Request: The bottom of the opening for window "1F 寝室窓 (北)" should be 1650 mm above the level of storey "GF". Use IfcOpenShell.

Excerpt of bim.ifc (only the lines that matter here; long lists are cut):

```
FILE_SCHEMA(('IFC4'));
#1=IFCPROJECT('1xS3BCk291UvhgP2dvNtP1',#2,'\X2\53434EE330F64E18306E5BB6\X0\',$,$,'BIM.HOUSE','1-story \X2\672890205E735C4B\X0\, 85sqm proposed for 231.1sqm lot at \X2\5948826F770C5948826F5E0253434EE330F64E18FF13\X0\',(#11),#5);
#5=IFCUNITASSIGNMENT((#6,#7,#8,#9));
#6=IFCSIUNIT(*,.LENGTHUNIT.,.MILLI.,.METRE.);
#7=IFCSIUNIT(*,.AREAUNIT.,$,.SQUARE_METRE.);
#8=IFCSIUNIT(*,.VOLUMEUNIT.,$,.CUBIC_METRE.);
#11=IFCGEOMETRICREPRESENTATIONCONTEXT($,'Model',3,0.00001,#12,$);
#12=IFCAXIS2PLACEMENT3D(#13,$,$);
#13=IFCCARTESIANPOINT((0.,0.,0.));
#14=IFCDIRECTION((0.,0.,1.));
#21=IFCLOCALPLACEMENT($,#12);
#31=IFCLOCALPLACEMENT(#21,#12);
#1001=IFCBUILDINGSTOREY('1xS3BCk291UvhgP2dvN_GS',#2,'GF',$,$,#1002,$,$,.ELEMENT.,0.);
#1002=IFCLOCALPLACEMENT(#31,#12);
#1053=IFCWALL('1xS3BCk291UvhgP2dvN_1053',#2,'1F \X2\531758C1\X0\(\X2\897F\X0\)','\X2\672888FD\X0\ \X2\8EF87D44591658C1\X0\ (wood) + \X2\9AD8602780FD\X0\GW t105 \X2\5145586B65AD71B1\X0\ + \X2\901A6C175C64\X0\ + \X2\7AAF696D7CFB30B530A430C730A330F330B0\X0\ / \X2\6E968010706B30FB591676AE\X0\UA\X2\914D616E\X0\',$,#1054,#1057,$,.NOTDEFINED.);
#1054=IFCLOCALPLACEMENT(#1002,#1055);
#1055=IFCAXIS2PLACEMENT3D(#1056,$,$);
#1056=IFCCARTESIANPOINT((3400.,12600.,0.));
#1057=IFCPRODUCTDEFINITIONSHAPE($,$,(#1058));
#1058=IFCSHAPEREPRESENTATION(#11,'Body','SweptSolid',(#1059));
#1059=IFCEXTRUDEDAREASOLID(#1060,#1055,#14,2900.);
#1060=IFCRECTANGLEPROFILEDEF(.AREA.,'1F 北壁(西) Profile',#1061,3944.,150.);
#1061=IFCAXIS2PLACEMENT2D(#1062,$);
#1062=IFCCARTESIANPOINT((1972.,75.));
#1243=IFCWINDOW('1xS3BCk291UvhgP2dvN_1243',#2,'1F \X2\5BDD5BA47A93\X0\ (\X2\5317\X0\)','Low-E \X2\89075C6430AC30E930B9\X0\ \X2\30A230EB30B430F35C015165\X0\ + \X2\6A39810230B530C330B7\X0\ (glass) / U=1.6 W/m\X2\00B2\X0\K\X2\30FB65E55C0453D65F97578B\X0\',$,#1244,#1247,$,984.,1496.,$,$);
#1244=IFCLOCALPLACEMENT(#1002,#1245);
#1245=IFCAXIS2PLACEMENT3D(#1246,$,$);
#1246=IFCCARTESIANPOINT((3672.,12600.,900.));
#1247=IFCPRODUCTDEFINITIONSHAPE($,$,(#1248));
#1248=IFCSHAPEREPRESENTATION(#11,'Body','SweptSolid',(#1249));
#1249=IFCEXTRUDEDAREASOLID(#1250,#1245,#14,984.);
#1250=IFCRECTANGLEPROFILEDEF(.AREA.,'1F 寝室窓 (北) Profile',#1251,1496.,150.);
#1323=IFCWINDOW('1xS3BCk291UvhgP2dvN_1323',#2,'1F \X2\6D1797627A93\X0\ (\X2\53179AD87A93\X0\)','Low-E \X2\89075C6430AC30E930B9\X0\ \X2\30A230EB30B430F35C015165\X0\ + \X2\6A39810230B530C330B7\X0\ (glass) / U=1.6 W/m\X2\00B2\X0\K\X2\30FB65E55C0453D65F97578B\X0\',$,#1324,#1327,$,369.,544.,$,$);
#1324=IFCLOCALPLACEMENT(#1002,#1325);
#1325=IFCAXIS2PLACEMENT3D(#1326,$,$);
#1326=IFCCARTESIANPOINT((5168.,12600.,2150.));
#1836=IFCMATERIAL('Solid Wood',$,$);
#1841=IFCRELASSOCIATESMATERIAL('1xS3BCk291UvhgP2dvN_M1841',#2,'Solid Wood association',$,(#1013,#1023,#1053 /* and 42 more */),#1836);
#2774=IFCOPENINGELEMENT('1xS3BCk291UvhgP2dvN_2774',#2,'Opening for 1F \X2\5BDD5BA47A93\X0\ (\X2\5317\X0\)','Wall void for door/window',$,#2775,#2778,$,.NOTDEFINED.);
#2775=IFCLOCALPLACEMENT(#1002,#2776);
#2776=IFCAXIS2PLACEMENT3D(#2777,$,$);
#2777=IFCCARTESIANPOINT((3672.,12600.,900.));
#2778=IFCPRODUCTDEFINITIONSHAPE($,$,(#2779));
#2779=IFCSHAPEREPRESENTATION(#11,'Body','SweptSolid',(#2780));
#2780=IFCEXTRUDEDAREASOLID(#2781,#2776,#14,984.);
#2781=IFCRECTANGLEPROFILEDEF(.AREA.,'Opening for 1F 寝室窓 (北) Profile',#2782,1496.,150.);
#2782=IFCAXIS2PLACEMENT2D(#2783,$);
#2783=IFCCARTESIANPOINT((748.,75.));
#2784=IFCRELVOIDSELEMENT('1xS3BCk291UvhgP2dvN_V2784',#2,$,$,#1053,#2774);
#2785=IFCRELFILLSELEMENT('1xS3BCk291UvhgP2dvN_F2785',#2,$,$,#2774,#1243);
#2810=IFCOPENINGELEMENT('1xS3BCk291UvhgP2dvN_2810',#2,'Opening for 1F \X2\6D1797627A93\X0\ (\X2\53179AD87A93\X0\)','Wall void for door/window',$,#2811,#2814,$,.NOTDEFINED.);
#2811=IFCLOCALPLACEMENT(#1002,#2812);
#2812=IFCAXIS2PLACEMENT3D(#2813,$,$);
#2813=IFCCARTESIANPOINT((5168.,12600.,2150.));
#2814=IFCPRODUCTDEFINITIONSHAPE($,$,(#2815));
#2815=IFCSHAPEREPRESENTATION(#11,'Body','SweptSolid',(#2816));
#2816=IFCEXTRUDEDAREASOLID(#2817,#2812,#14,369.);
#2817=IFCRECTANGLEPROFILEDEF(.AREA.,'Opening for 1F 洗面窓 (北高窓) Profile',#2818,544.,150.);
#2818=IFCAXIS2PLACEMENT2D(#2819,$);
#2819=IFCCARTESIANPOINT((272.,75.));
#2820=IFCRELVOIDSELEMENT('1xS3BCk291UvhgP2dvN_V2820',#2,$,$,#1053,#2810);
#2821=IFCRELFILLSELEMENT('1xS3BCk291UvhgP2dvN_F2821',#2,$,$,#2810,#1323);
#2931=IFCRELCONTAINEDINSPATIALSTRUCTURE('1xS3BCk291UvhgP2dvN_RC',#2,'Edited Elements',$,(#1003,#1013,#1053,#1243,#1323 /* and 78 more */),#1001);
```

```python
import numpy as np
import ifcopenshell
import ifcopenshell.api.geometry
import ifcopenshell.geom
import ifcopenshell.util.element
import ifcopenshell.util.placement
import ifcopenshell.util.shape
import ifcopenshell.util.unit

model = ifcopenshell.open("bim.ifc")
unit_scale = ifcopenshell.util.unit.calculate_unit_scale(model)

window = model.by_guid("1xS3BCk291UvhgP2dvN_1243")
opening = window.FillsVoids[0].RelatingOpeningElement
storey = ifcopenshell.util.element.get_container(window, ifc_class="IfcBuildingStorey")
level = ifcopenshell.util.placement.get_local_placement(storey.ObjectPlacement)[2, 3]

# The opening's origin need not be at the sill, so measure its lowest point.
shape = ifcopenshell.geom.create_shape(ifcopenshell.geom.settings(), opening)
bottom = ifcopenshell.util.shape.get_shape_bottom_elevation(shape, shape.geometry) / unit_scale
dz = level + 1650.0 - bottom

shift = np.array([0.0, 0.0, dz])
# The window is not placed relative to its opening, so move both.
for product in (opening, window):
    matrix = ifcopenshell.util.placement.get_local_placement(product.ObjectPlacement)
    matrix[:3, 3] += shift
    ifcopenshell.api.geometry.edit_object_placement(model, product=product, matrix=matrix, is_si=False)

print(f"moved by {dz * unit_scale:+.3f} m")

model.write("bim_rev.ifc")
```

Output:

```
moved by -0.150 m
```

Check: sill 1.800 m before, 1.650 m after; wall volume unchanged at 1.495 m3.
